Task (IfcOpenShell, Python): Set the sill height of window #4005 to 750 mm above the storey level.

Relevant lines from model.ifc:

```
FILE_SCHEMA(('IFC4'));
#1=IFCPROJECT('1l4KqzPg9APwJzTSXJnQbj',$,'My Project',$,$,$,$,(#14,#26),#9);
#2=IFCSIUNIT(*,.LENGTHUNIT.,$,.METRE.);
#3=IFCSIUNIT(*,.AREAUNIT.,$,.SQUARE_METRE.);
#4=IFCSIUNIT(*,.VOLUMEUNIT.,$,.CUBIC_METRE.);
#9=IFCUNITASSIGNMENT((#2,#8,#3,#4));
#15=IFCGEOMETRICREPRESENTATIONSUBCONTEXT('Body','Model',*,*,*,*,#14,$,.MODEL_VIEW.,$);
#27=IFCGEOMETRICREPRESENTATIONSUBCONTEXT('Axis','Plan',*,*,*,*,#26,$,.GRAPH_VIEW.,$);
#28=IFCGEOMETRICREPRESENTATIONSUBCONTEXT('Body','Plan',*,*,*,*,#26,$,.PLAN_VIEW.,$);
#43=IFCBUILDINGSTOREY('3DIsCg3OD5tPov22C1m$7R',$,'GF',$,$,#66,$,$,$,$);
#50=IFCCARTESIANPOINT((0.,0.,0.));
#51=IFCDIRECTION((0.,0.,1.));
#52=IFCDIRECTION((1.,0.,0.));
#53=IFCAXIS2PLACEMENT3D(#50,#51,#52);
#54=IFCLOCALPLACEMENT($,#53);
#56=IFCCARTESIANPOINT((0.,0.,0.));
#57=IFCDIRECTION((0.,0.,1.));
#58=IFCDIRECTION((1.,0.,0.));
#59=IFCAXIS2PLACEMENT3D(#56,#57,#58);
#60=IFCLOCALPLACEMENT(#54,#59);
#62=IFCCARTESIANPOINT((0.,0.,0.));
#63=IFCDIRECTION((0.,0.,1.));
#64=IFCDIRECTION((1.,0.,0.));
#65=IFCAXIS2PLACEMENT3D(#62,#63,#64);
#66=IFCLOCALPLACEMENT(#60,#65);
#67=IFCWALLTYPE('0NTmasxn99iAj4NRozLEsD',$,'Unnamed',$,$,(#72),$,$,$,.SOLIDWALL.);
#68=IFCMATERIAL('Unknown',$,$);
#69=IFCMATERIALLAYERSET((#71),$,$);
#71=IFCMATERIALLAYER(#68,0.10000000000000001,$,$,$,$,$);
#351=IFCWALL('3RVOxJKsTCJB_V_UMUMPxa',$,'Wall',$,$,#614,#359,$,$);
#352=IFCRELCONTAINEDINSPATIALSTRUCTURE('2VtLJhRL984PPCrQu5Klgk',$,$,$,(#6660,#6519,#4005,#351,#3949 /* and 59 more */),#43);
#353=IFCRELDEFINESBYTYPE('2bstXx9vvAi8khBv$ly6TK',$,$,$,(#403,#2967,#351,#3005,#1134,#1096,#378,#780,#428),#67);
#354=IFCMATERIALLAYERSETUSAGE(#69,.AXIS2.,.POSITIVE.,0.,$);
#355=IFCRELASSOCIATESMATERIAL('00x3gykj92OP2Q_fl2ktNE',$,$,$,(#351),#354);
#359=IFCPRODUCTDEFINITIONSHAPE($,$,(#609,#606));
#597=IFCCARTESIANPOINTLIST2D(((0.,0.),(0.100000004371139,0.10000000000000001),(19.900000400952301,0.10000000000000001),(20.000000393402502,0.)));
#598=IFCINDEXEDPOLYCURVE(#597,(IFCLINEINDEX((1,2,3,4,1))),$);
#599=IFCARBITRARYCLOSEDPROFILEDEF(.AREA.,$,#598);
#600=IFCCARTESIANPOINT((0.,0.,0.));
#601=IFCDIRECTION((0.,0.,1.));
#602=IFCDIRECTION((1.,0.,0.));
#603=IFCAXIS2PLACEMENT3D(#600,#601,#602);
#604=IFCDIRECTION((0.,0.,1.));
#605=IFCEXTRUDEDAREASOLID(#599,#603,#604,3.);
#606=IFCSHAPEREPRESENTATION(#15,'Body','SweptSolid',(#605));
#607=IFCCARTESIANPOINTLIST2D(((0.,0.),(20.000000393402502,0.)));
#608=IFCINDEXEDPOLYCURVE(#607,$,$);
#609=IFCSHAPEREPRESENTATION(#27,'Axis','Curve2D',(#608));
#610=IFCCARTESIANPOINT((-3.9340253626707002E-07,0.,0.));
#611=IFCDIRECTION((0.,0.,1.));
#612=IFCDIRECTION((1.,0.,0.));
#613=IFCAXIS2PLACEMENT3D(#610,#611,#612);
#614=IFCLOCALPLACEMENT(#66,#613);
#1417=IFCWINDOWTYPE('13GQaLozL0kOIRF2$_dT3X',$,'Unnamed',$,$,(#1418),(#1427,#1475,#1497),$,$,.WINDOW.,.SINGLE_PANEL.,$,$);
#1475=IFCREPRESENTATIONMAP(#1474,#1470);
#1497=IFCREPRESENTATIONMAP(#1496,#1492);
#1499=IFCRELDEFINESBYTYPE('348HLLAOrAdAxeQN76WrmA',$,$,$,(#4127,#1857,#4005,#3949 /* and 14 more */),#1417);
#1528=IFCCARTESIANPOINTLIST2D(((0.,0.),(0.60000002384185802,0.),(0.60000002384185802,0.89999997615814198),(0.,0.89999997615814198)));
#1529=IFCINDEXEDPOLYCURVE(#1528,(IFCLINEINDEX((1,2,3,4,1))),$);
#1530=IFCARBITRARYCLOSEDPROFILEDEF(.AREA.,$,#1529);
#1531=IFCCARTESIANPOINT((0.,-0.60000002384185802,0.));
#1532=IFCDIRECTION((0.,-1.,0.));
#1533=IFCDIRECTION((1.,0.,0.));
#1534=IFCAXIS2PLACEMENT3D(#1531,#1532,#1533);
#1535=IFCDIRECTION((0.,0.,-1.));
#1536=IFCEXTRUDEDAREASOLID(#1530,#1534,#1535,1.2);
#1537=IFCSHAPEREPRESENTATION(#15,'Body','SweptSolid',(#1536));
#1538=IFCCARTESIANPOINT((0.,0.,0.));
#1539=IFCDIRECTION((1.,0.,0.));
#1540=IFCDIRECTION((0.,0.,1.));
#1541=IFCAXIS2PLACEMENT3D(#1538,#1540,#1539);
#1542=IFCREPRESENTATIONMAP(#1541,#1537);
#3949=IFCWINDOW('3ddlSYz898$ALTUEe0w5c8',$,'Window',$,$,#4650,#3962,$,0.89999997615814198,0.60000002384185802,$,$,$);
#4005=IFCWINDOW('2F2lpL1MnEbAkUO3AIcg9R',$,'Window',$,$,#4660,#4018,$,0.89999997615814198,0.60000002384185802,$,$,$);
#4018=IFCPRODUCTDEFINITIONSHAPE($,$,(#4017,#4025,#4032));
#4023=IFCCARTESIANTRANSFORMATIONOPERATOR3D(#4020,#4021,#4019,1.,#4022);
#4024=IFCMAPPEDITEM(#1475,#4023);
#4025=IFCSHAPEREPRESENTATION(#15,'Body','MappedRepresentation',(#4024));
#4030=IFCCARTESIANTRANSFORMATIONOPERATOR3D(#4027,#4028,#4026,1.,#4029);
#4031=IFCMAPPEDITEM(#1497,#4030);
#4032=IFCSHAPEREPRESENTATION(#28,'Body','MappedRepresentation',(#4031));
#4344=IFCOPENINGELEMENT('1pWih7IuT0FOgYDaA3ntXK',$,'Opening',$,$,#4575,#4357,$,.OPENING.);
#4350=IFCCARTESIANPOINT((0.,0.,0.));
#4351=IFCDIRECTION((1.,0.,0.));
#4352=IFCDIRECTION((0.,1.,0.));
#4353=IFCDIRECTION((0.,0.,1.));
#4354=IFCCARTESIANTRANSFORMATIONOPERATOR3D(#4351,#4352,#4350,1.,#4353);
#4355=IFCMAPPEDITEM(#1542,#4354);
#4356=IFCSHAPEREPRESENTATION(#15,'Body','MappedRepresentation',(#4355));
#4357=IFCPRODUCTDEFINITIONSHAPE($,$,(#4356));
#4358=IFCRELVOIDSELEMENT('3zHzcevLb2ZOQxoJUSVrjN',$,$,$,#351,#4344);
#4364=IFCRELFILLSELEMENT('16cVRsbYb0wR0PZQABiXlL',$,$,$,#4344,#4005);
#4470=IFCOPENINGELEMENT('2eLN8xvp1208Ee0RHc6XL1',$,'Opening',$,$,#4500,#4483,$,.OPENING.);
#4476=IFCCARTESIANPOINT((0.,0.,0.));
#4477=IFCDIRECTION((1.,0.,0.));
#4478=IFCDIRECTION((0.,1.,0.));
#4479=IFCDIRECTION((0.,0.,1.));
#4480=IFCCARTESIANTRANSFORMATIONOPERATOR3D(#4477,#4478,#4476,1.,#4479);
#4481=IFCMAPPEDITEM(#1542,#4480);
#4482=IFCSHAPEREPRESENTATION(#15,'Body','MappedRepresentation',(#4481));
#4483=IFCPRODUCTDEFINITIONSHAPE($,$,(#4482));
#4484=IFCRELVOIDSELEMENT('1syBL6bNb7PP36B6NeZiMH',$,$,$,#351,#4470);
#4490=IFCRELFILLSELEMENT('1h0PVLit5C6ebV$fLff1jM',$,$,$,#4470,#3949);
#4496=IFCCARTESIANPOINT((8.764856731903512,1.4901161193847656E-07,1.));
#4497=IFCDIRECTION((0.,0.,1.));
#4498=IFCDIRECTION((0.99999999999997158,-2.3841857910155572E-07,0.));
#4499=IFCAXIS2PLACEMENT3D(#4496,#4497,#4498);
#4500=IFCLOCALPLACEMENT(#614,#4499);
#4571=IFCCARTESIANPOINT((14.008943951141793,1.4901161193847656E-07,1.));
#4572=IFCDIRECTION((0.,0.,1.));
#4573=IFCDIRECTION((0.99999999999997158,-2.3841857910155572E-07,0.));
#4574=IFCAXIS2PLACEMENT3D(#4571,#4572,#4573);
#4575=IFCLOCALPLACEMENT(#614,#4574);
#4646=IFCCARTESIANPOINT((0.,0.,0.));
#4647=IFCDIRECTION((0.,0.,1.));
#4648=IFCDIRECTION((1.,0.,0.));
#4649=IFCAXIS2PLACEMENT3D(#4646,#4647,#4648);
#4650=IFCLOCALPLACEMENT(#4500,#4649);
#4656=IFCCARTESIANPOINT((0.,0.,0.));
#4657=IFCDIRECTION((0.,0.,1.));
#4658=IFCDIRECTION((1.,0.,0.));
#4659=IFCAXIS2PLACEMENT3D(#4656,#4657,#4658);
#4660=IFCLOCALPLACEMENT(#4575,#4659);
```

```python
import numpy as np
import ifcopenshell
import ifcopenshell.api.geometry
import ifcopenshell.geom
import ifcopenshell.util.element
import ifcopenshell.util.placement
import ifcopenshell.util.shape
import ifcopenshell.util.unit

model = ifcopenshell.open("model.ifc")
unit_scale = ifcopenshell.util.unit.calculate_unit_scale(model)

window = model.by_guid("2F2lpL1MnEbAkUO3AIcg9R")
opening = window.FillsVoids[0].RelatingOpeningElement
storey = ifcopenshell.util.element.get_container(window, ifc_class="IfcBuildingStorey")
level = ifcopenshell.util.placement.get_local_placement(storey.ObjectPlacement)[2, 3]

# The opening's origin need not be at the sill, so measure its lowest point.
shape = ifcopenshell.geom.create_shape(ifcopenshell.geom.settings(), opening)
bottom = ifcopenshell.util.shape.get_shape_bottom_elevation(shape, shape.geometry) / unit_scale
dz = level + 0.75 / unit_scale - bottom

shift = np.array([0.0, 0.0, dz])
# The window is placed relative to its opening, so it follows when the opening moves.
matrix = ifcopenshell.util.placement.get_local_placement(opening.ObjectPlacement)
matrix[:3, 3] += shift
ifcopenshell.api.geometry.edit_object_placement(
    model, product=opening, matrix=matrix, is_si=False, should_transform_children=True
)

print(f"moved by {dz * unit_scale:+.3f} m")

model.write("model_updated.ifc")
```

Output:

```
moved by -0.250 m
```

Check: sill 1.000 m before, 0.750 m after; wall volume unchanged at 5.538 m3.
